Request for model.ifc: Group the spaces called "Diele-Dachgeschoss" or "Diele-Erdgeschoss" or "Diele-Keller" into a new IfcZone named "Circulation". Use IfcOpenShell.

First a look at what the model holds.

```python
import ifcopenshell

model = ifcopenshell.open("model.ifc")
print(model.schema)
seen = {}
for space in model.by_type("IfcSpace"):
    seen[space.LongName] = seen.get(space.LongName, 0) + 1
for name, count in sorted(seen.items(), key=str):
    print(count, "x", name)
print("zones:", [z.Name for z in model.by_type("IfcZone")][:20])
```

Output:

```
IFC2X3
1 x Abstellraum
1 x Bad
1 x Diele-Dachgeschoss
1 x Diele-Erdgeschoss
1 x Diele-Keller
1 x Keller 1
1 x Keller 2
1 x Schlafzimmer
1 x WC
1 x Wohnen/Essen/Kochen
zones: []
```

```python
import ifcopenshell
import ifcopenshell.api.group
import ifcopenshell.api.root

model = ifcopenshell.open("model.ifc")

names = {"Diele-Dachgeschoss", "Diele-Erdgeschoss", "Diele-Keller"}
spaces = [s for s in model.by_type("IfcSpace") if s.LongName in names]

zone = ifcopenshell.api.root.create_entity(model, ifc_class="IfcZone", name="Circulation")
ifcopenshell.api.group.assign_group(model, products=spaces, group=zone)
print(len(spaces), "spaces in", zone.Name)

model.write("model_rev.ifc")
```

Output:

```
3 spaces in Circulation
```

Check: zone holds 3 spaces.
